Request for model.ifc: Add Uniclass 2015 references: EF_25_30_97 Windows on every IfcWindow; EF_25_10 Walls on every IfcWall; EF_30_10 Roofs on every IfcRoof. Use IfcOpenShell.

First a look at what the model holds.

```python
import ifcopenshell

model = ifcopenshell.open("model.ifc")
print(model.schema)
print("classifications:", [c.Name for c in model.by_type("IfcClassification")])
for ifc_class in ("IfcDoor", "IfcRoof", "IfcStair", "IfcWall", "IfcWindow"):
    print(ifc_class, len(model.by_type(ifc_class)))
```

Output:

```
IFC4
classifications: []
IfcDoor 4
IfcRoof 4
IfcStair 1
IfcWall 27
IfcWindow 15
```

```python
import ifcopenshell
import ifcopenshell.api.classification

model = ifcopenshell.open("model.ifc")

system = ifcopenshell.api.classification.add_classification(model, classification="Uniclass 2015")

codes = {
    "IfcWindow": ("EF_25_30_97", "Windows"),
    "IfcWall": ("EF_25_10", "Walls"),
    "IfcRoof": ("EF_30_10", "Roofs"),
}
for ifc_class, (code, name) in codes.items():
    products = model.by_type(ifc_class)
    ifcopenshell.api.classification.add_reference(
        model, products=products, classification=system, identification=code, name=name
    )
    print(code, len(products))

model.write("model_rev.ifc")
```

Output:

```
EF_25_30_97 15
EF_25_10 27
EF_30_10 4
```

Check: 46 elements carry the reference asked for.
